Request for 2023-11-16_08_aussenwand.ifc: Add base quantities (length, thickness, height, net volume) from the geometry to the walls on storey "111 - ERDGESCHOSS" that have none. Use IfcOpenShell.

First a look at what the model holds.

```python
import ifcopenshell
import ifcopenshell.util.element
import ifcopenshell.util.unit

model = ifcopenshell.open("2023-11-16_08_aussenwand.ifc")
print(model.schema)
for unit_type in ("LENGTHUNIT", "AREAUNIT", "VOLUMEUNIT"):
    print(unit_type, ifcopenshell.util.unit.calculate_unit_scale(model, unit_type))
storey = next(s for s in model.by_type("IfcBuildingStorey") if s.Name == "111 - ERDGESCHOSS")
walls = [e for e in ifcopenshell.util.element.get_decomposition(storey) if e.is_a("IfcWall")]
for e in sorted(walls, key=lambda e: e.id()):
    print(e.id(), e.is_a(), e.Name, list(ifcopenshell.util.element.get_psets(e, qtos_only=True)), sep=" | ")
```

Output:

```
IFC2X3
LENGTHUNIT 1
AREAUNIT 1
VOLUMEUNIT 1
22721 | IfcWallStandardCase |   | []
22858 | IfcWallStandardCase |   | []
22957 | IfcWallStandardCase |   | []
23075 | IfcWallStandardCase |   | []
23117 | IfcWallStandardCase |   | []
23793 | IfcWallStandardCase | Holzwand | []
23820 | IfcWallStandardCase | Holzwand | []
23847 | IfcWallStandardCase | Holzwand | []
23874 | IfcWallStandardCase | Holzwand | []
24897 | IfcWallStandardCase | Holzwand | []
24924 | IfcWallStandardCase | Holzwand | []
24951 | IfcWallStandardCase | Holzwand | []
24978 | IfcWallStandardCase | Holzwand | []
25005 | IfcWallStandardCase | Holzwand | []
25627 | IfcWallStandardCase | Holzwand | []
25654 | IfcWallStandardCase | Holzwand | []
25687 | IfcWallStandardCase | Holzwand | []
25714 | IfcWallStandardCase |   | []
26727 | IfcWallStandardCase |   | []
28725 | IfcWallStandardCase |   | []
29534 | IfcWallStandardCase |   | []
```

```python
import ifcopenshell
import ifcopenshell.api.pset
import ifcopenshell.geom
import ifcopenshell.util.element
import ifcopenshell.util.shape
import ifcopenshell.util.unit

model = ifcopenshell.open("2023-11-16_08_aussenwand.ifc")
unit_scale = ifcopenshell.util.unit.calculate_unit_scale(model)
volume_scale = ifcopenshell.util.unit.calculate_unit_scale(model, "VOLUMEUNIT")
settings = ifcopenshell.geom.settings()

storey = next(s for s in model.by_type("IfcBuildingStorey") if s.Name == "111 - ERDGESCHOSS")
walls = [e for e in ifcopenshell.util.element.get_decomposition(storey) if e.is_a("IfcWall")]

for e in sorted(walls, key=lambda e: e.id()):
    if ifcopenshell.util.element.get_psets(e, qtos_only=True, should_inherit=False):
        continue
    # Geometry comes back in metres, in the element's own axes.
    shape = ifcopenshell.geom.create_shape(settings, e)
    values = {
        "Length": ifcopenshell.util.shape.get_x(shape.geometry) / unit_scale,
        "Width": ifcopenshell.util.shape.get_y(shape.geometry) / unit_scale,
        "Height": ifcopenshell.util.shape.get_z(shape.geometry) / unit_scale,
        "NetVolume": ifcopenshell.util.shape.get_volume(shape.geometry) / volume_scale,
    }
    qto = ifcopenshell.api.pset.add_qto(model, product=e, name="BaseQuantities")
    ifcopenshell.api.pset.edit_qto(model, qto=qto, properties=values)
    print(e.id(), {k: round(v, 3) for k, v in values.items()})

model.write("2023-11-16_08_aussenwand_edited.ifc")
```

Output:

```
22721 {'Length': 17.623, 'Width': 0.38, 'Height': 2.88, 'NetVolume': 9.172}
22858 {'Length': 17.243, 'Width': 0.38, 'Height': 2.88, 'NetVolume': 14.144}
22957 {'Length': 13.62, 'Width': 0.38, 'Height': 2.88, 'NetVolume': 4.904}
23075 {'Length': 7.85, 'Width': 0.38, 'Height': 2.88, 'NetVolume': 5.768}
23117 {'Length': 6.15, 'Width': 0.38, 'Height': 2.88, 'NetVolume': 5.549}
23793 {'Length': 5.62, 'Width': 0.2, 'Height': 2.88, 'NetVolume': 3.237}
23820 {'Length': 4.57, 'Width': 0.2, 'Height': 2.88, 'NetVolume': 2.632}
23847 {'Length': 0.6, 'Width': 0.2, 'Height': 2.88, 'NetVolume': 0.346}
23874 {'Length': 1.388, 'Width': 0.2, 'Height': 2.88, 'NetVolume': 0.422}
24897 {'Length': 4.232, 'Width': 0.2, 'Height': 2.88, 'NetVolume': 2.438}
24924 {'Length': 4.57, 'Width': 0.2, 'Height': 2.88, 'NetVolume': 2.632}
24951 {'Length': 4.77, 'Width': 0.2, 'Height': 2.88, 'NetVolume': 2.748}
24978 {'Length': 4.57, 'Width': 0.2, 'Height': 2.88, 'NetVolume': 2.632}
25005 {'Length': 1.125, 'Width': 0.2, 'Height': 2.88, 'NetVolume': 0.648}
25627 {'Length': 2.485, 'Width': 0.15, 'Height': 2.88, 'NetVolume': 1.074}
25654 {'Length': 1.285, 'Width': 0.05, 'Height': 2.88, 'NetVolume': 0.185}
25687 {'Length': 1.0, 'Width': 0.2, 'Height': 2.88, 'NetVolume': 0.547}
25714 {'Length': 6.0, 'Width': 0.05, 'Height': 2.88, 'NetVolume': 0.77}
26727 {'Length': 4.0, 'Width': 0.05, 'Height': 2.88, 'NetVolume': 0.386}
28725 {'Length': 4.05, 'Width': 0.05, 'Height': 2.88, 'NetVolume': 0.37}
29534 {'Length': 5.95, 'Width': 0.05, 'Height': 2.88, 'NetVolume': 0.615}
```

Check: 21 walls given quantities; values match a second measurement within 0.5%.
